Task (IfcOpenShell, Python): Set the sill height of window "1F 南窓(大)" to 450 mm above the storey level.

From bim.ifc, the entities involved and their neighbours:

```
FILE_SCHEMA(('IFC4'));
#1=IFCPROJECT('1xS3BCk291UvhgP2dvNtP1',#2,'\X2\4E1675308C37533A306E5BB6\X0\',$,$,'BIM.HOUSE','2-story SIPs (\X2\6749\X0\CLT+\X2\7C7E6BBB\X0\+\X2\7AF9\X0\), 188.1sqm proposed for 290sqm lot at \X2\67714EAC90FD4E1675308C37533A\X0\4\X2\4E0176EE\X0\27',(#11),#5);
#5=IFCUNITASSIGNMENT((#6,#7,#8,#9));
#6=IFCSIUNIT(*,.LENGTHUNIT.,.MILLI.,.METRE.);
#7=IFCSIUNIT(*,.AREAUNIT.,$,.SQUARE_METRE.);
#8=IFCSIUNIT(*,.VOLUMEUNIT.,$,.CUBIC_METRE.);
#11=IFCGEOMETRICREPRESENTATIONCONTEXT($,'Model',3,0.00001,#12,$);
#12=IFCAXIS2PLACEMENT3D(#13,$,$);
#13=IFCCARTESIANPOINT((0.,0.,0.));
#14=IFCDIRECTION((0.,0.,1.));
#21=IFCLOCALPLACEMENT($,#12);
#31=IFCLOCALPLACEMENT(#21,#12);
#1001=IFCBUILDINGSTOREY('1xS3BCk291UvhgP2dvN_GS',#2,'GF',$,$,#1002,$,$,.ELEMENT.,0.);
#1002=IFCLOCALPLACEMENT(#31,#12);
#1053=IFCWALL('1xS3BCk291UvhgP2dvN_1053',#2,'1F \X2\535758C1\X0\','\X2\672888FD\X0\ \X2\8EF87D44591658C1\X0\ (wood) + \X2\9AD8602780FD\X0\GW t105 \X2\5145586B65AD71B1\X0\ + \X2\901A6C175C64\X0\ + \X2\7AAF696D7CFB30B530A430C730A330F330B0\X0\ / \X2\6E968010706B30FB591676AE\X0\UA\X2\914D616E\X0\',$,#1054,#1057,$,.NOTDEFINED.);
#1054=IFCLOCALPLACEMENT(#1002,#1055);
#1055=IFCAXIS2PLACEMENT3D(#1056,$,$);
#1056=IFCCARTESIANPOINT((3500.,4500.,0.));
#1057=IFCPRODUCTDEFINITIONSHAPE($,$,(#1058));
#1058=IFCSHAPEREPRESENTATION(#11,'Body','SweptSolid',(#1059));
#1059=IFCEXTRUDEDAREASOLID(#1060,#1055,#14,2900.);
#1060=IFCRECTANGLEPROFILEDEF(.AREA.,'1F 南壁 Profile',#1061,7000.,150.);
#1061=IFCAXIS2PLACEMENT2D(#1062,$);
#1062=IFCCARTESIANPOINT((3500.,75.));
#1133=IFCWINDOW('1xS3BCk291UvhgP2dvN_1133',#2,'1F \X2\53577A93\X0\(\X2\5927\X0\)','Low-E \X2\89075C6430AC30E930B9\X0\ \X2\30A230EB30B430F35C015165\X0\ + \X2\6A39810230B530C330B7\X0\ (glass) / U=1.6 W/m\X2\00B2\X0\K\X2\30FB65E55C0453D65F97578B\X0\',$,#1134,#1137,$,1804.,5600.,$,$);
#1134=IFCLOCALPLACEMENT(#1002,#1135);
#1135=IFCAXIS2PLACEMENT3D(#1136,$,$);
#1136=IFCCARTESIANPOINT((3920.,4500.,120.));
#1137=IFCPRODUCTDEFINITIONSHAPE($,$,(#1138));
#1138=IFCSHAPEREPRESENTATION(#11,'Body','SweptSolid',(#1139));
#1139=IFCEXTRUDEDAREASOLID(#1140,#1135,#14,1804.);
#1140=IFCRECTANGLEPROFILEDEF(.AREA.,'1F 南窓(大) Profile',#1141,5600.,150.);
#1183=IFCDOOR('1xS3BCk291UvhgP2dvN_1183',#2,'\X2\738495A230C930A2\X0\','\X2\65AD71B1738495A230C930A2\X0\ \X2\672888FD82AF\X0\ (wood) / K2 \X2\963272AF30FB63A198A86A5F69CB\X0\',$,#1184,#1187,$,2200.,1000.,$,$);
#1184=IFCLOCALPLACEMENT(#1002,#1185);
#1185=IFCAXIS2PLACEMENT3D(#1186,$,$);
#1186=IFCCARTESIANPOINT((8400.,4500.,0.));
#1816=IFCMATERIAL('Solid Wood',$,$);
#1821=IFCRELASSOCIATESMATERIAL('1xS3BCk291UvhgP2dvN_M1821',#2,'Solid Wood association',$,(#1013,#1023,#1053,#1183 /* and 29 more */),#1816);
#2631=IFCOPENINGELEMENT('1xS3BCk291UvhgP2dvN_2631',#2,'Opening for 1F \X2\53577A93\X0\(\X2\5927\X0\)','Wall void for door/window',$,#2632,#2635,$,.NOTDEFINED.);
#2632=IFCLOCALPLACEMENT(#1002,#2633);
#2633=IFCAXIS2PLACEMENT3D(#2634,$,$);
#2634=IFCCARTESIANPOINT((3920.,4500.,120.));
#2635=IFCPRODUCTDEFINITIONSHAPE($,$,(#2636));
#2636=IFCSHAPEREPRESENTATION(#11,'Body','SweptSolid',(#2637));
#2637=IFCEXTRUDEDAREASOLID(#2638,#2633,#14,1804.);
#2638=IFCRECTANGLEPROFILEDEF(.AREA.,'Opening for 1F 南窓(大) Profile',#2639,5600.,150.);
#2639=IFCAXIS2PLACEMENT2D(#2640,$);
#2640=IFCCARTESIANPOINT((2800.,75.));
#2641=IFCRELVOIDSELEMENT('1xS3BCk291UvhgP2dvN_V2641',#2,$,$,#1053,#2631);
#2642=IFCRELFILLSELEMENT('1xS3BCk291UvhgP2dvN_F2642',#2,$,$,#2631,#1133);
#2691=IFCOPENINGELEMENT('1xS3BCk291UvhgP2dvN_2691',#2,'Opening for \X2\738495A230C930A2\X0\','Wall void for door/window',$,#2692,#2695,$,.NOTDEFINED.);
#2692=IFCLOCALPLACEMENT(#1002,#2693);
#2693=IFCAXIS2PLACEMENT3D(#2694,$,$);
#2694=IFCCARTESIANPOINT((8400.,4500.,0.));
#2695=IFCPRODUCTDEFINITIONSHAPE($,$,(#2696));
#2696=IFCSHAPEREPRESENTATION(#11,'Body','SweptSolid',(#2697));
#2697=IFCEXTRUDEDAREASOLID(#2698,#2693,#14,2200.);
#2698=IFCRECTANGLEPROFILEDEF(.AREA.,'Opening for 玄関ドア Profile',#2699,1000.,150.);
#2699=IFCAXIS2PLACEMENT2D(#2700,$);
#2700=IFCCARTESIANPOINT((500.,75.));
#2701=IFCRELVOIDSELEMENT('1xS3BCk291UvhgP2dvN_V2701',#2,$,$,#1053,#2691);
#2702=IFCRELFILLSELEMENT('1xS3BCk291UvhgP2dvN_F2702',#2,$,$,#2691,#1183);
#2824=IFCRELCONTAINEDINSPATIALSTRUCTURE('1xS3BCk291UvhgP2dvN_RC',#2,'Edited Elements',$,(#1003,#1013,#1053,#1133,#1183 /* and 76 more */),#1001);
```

```python
import numpy as np
import ifcopenshell
import ifcopenshell.api.geometry
import ifcopenshell.geom
import ifcopenshell.util.element
import ifcopenshell.util.placement
import ifcopenshell.util.shape
import ifcopenshell.util.unit

model = ifcopenshell.open("bim.ifc")
unit_scale = ifcopenshell.util.unit.calculate_unit_scale(model)

window = model.by_id(1133)
opening = window.FillsVoids[0].RelatingOpeningElement
storey = ifcopenshell.util.element.get_container(window, ifc_class="IfcBuildingStorey")
level = ifcopenshell.util.placement.get_local_placement(storey.ObjectPlacement)[2, 3]

# The opening's origin need not be at the sill, so measure its lowest point.
shape = ifcopenshell.geom.create_shape(ifcopenshell.geom.settings(), opening)
bottom = ifcopenshell.util.shape.get_shape_bottom_elevation(shape, shape.geometry) / unit_scale
dz = level + 450.0 - bottom

shift = np.array([0.0, 0.0, dz])
# The window is not placed relative to its opening, so move both.
for product in (opening, window):
    matrix = ifcopenshell.util.placement.get_local_placement(product.ObjectPlacement)
    matrix[:3, 3] += shift
    ifcopenshell.api.geometry.edit_object_placement(model, product=product, matrix=matrix, is_si=False)

print(f"moved by {dz * unit_scale:+.3f} m")

model.write("bim-out.ifc")
```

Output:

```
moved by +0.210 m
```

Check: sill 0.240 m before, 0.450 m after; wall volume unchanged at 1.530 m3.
